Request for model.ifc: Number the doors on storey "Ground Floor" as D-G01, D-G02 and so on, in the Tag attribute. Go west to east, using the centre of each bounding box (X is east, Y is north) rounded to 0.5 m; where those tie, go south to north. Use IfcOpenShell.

First a look at what the model holds.

```python
import ifcopenshell
import ifcopenshell.util.element
import ifcopenshell.util.placement

model = ifcopenshell.open("model.ifc")
print(model.schema)
storey = next(s for s in model.by_type("IfcBuildingStorey") if s.Name == "Ground Floor")
doors = [e for e in ifcopenshell.util.element.get_decomposition(storey) if e.is_a("IfcDoor")]
for e in sorted(doors, key=lambda e: e.id()):
    origin = ifcopenshell.util.placement.get_local_placement(e.ObjectPlacement)[:3, 3]
    print(e.id(), e.Tag, e.Name, origin.round(2) + 0.0, sep=" | ")
```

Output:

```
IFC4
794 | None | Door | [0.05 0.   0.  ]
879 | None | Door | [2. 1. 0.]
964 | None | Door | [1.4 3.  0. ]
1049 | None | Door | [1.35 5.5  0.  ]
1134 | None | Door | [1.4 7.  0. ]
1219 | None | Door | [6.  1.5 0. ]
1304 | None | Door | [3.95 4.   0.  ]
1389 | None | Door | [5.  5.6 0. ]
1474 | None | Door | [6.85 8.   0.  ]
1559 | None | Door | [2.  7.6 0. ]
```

```python
import ifcopenshell
import ifcopenshell.geom
import ifcopenshell.util.element
import ifcopenshell.util.shape

model = ifcopenshell.open("model.ifc")
settings = ifcopenshell.geom.settings()
settings.set("use-world-coords", True)


def centre(element):
    shape = ifcopenshell.geom.create_shape(settings, element)
    return ifcopenshell.util.shape.get_bbox_centroid(shape.geometry)


storey = next(s for s in model.by_type("IfcBuildingStorey") if s.Name == "Ground Floor")
doors = [e for e in ifcopenshell.util.element.get_decomposition(storey) if e.is_a("IfcDoor")]

# Insertion points can sit at a corner or the storey origin, so sort by the geometry (in metres).
centres = {e: centre(e) for e in doors}
doors.sort(key=lambda e: (round(centres[e][0] / 0.5), centres[e][1]))

for i, e in enumerate(doors, start=1):
    number = f"D-G{i:02d}"
    e.Tag = number
    print(e.id(), number)

model.write("model_v2.ifc")
```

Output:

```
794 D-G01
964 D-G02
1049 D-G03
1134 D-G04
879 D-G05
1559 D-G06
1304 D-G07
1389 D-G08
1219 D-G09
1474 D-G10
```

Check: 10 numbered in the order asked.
